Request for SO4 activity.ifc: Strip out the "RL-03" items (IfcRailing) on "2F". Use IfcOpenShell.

First a look at what the model holds.

```python
import ifcopenshell
import ifcopenshell.util.element

model = ifcopenshell.open("SO4 activity.ifc")
print(model.schema)
storey = next(s for s in model.by_type("IfcBuildingStorey") if s.Name == "2F")
railings = [e for e in ifcopenshell.util.element.get_decomposition(storey) if e.is_a("IfcRailing")]
seen = {}
for e in railings:
    element_type = ifcopenshell.util.element.get_type(e)
    name = element_type.Name if element_type not in (None, e) else None
    seen[name] = seen.get(name, 0) + 1
for name, count in sorted(seen.items(), key=str):
    print(count, "x", name)
```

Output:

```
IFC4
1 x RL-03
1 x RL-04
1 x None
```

```python
import ifcopenshell
import ifcopenshell.api.root
import ifcopenshell.util.element

model = ifcopenshell.open("SO4 activity.ifc")

storey = next(s for s in model.by_type("IfcBuildingStorey") if s.Name == "2F")
railings = [e for e in ifcopenshell.util.element.get_decomposition(storey) if e.is_a("IfcRailing")]
targets = [e for e in railings if (t := ifcopenshell.util.element.get_type(e)) not in (None, e) and t.Name == "RL-03"]

for e in targets:
    ifcopenshell.api.root.remove_product(model, product=e)
print(len(targets), "removed")

model.write("SO4 activity_edited.ifc")
```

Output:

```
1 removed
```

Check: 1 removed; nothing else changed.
